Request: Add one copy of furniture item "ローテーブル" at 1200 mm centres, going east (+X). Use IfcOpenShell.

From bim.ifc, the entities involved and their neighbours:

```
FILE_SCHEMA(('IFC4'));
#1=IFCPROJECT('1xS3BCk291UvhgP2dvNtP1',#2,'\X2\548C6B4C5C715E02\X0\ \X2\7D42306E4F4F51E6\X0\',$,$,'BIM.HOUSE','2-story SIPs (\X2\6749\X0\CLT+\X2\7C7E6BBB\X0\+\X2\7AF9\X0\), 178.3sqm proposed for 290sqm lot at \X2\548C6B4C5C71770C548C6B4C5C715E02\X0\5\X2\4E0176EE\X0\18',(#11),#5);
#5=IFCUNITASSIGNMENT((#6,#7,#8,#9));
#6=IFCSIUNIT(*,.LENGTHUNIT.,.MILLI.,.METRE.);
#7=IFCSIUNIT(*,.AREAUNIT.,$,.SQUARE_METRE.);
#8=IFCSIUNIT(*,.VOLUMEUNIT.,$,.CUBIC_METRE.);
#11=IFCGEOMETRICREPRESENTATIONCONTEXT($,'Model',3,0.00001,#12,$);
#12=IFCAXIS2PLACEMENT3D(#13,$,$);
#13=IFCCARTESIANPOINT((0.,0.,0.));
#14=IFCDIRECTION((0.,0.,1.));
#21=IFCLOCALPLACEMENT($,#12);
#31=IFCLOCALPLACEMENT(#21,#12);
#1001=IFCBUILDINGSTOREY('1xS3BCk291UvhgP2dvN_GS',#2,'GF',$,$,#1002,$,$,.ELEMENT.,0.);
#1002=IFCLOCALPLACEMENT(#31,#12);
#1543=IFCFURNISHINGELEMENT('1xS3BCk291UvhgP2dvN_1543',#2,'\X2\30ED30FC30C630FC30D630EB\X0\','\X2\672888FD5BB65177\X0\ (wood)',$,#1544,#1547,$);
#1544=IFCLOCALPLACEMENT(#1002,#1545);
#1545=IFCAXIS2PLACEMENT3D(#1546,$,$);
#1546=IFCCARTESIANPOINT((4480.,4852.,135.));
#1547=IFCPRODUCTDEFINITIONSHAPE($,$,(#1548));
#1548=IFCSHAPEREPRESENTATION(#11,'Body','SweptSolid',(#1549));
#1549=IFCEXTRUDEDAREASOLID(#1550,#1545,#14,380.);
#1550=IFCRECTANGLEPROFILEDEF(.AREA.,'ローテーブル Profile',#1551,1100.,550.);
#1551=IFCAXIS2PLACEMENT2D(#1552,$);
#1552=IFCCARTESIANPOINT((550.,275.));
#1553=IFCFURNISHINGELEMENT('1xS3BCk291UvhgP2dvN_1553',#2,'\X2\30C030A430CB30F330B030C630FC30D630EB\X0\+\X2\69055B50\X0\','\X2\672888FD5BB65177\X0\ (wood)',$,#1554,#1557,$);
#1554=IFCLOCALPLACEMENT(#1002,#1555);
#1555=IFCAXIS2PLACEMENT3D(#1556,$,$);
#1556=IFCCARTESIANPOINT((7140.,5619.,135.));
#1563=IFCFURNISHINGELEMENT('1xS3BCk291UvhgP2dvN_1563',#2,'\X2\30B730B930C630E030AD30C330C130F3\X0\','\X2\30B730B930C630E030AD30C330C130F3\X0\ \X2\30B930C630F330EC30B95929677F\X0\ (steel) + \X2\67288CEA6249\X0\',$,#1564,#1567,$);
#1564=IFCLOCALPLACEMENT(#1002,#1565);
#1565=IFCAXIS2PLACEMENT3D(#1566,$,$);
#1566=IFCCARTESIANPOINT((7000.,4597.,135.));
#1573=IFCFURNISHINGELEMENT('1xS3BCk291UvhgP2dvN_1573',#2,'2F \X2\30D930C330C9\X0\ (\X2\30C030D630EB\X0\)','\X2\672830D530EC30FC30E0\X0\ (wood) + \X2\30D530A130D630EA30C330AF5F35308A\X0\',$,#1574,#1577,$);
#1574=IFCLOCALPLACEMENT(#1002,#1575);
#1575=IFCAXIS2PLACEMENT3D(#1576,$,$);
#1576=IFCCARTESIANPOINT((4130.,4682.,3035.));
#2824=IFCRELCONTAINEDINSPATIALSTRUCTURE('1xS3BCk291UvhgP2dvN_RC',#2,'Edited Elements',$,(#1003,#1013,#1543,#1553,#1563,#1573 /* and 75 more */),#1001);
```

```python
import numpy as np
import ifcopenshell
import ifcopenshell.api.geometry
import ifcopenshell.api.root
import ifcopenshell.util.element
import ifcopenshell.util.placement

model = ifcopenshell.open("bim.ifc")


def reuse_history(source, copy):
    """copy_class also copies each property set's owner history, people and application; keep the originals."""
    for rel in copy.IsDefinedBy:
        if rel.is_a("IfcRelDefinesByProperties") and (history := rel.RelatingPropertyDefinition.OwnerHistory):
            rel.RelatingPropertyDefinition.OwnerHistory = source.OwnerHistory
            ifcopenshell.util.element.remove_deep2(model, history)


source = model.by_id(1543)
base = ifcopenshell.util.placement.get_local_placement(source.ObjectPlacement)
step = np.array([1.0, 0.0, 0.0]) * 1200.0

for i in range(1, 2):
    copy = ifcopenshell.api.root.copy_class(model, product=source)
    copy.Representation = ifcopenshell.util.element.copy_deep(
        model, source.Representation, exclude=["IfcGeometricRepresentationContext", "IfcRepresentationMap"]
    )
    reuse_history(source, copy)
    matrix = base.copy()
    matrix[:3, 3] += i * step
    print("added at", matrix[:3, 3].round(3) + 0.0)
    ifcopenshell.api.geometry.edit_object_placement(model, product=copy, matrix=matrix, is_si=False)

model.write("bim_edited.ifc")
```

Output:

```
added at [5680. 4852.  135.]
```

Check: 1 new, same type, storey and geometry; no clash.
